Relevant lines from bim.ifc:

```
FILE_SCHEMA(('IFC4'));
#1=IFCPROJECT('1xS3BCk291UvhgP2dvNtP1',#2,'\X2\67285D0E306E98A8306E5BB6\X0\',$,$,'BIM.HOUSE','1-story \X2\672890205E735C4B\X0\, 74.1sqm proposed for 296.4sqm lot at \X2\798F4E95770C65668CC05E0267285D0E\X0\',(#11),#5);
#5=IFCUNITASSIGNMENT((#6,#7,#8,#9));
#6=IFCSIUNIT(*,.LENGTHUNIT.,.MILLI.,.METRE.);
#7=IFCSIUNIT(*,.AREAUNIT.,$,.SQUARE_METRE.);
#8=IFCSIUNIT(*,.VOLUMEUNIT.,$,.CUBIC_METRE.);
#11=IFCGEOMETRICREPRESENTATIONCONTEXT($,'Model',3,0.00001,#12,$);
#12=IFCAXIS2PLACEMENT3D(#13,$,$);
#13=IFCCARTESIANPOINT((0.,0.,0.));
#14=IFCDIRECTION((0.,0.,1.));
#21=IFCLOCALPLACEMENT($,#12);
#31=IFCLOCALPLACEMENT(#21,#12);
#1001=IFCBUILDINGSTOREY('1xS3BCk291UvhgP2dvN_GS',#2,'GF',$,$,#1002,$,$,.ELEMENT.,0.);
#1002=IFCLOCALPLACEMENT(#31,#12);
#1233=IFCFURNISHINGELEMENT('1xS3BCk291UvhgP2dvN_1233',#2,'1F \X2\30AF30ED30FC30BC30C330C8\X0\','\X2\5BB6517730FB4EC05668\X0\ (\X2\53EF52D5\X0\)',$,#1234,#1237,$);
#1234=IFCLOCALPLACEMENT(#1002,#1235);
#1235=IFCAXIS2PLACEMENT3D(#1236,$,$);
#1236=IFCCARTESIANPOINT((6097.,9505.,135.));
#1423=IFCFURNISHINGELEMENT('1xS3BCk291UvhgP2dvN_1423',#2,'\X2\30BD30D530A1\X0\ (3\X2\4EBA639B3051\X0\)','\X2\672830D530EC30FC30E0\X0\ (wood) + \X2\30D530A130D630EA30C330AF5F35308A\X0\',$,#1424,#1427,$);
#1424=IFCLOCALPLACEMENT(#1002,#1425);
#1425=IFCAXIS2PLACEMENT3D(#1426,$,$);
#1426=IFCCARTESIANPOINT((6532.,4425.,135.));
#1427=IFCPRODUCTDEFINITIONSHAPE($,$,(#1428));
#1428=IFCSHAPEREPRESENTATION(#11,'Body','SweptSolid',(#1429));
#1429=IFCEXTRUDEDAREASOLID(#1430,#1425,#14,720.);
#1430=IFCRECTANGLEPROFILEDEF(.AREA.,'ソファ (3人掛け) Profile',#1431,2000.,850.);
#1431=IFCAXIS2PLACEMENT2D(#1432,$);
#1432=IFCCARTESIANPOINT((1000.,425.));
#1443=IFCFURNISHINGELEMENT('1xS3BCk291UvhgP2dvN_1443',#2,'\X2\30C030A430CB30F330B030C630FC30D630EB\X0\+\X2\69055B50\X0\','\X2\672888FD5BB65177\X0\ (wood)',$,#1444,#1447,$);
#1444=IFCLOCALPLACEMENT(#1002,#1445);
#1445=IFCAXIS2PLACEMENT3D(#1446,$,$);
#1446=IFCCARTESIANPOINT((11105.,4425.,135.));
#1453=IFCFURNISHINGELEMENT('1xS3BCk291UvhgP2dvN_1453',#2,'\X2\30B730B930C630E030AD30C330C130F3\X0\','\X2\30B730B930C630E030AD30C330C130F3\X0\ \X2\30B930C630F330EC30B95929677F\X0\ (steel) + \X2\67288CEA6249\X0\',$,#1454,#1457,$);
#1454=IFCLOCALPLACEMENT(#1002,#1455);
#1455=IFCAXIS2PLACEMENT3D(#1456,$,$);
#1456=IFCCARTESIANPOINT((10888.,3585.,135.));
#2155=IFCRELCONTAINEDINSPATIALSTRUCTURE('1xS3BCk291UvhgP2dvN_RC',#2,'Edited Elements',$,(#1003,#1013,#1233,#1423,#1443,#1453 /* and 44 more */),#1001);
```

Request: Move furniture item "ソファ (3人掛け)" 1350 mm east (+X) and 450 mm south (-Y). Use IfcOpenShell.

```python
import ifcopenshell
import ifcopenshell.api.geometry
import ifcopenshell.util.placement

model = ifcopenshell.open("bim.ifc")

item = model.by_guid("1xS3BCk291UvhgP2dvN_1423")
matrix = ifcopenshell.util.placement.get_local_placement(item.ObjectPlacement)
matrix[0, 3] += 1350.0
matrix[1, 3] -= 450.0
ifcopenshell.api.geometry.edit_object_placement(model, product=item, matrix=matrix, is_si=False)

print(ifcopenshell.util.placement.get_local_placement(item.ObjectPlacement).round(3) + 0.0)

model.write("bim_updated.ifc")
```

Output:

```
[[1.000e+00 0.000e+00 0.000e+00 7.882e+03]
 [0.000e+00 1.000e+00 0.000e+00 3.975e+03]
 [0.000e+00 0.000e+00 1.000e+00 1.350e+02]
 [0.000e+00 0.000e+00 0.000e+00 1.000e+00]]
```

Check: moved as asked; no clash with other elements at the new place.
